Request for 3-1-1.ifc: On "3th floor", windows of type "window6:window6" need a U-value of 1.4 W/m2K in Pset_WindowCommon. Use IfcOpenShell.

First a look at what the model holds.

```python
import ifcopenshell
import ifcopenshell.util.element

model = ifcopenshell.open("3-1-1.ifc")
print(model.schema)
storey = next(s for s in model.by_type("IfcBuildingStorey") if s.Name == "3th floor")
windows = [e for e in ifcopenshell.util.element.get_decomposition(storey) if e.is_a("IfcWindow")]
seen = {}
for e in windows:
    element_type = ifcopenshell.util.element.get_type(e)
    key = (element_type.Name if element_type != e and element_type else None, ifcopenshell.util.element.get_pset(e, "Pset_WindowCommon", "ThermalTransmittance"))
    seen[key] = seen.get(key, 0) + 1
for (name, value), count in sorted(seen.items(), key=str):
    print(count, "x", name, "|", value)
```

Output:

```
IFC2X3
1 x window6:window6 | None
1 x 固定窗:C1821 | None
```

```python
import ifcopenshell
import ifcopenshell.api.pset
import ifcopenshell.util.element

model = ifcopenshell.open("3-1-1.ifc")

storey = next(s for s in model.by_type("IfcBuildingStorey") if s.Name == "3th floor")
windows = [e for e in ifcopenshell.util.element.get_decomposition(storey) if e.is_a("IfcWindow")]

count = 0
for e in windows:
    element_type = ifcopenshell.util.element.get_type(e)
    if element_type in (None, e) or element_type.Name != "window6:window6":
        continue
    # add_pset returns the element's existing set when there is one.
    pset = ifcopenshell.api.pset.add_pset(model, product=e, name="Pset_WindowCommon")
    ifcopenshell.api.pset.edit_pset(model, pset=pset, properties={"ThermalTransmittance": 1.4})
    count += 1

print(count, "windows updated")

model.write("3-1-1_v2.ifc")
```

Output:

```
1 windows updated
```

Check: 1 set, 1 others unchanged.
